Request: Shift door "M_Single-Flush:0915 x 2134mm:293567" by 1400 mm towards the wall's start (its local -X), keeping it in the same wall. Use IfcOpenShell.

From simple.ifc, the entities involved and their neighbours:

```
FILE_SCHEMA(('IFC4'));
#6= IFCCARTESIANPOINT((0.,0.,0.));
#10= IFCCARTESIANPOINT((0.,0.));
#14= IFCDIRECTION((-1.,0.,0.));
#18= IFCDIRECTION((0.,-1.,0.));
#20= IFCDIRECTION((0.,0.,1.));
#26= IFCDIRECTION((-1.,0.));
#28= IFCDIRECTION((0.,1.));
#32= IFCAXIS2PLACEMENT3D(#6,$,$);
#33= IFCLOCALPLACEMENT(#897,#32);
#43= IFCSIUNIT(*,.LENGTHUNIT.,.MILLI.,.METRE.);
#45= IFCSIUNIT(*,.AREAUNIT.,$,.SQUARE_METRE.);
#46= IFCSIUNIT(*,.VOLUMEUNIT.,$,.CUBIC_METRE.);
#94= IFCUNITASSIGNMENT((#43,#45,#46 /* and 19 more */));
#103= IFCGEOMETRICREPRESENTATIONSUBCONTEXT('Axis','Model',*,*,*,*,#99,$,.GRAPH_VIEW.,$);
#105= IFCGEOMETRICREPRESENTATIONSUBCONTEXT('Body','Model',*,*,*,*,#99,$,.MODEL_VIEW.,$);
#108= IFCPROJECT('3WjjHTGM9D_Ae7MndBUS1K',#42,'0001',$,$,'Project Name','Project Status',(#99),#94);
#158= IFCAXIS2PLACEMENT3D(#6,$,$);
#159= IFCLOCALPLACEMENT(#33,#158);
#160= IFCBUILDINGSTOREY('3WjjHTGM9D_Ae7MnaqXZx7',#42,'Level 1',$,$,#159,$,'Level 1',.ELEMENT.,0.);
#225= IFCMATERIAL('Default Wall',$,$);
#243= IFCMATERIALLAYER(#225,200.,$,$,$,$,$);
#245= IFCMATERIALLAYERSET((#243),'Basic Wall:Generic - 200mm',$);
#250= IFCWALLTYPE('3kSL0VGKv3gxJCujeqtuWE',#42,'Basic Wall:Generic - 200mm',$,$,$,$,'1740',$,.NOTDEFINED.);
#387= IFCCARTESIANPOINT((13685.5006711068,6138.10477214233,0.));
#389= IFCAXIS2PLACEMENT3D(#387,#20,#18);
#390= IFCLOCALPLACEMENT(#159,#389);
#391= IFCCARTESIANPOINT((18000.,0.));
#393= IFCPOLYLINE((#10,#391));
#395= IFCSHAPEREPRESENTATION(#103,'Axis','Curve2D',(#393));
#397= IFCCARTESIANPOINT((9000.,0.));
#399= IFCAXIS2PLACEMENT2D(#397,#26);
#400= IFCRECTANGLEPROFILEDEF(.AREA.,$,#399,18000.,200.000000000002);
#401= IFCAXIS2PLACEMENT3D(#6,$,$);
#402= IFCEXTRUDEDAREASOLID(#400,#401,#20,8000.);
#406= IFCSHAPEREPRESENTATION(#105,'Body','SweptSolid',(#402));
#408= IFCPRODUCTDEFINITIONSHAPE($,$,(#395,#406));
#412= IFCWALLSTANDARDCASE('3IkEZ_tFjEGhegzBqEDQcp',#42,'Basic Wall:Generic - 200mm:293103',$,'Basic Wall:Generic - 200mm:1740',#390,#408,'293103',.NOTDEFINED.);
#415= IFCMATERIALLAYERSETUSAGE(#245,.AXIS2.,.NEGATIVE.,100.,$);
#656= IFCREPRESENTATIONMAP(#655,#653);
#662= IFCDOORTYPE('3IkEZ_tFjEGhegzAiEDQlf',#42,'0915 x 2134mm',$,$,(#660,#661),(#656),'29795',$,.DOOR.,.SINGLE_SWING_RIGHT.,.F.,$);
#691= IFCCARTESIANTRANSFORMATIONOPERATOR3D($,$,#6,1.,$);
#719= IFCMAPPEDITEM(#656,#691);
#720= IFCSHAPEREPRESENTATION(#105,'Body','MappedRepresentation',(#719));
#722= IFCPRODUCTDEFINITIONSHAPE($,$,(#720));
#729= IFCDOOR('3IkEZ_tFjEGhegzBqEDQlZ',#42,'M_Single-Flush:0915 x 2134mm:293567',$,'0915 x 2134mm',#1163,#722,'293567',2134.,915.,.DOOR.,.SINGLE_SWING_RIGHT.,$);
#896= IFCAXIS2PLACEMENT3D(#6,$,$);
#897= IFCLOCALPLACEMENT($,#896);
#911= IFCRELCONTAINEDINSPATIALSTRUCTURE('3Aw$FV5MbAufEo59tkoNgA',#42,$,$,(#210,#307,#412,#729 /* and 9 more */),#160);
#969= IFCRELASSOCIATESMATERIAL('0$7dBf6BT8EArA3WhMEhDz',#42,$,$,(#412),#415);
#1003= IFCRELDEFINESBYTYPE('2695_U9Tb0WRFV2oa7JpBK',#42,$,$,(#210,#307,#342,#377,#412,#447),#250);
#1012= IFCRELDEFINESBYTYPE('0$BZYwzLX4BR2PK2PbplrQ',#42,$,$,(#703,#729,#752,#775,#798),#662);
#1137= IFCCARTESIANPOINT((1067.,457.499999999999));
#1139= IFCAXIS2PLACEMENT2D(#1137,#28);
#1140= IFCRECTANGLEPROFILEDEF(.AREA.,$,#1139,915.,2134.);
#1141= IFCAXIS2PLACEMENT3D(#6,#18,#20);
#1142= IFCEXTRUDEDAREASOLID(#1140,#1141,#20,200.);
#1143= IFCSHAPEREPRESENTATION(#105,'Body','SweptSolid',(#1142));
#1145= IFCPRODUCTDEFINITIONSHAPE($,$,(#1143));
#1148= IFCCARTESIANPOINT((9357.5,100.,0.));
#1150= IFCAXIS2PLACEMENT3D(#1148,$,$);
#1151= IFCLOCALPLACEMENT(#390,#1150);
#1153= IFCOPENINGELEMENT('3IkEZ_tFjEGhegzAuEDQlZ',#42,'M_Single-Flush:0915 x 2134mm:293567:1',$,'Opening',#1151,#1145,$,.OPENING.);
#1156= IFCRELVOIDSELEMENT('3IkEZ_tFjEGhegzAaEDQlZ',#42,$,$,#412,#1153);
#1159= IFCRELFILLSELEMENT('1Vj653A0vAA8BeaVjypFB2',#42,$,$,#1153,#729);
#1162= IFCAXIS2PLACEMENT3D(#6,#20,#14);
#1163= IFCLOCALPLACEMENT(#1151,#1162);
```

```python
import ifcopenshell
import ifcopenshell.api.geometry
import ifcopenshell.util.placement
import ifcopenshell.util.unit

model = ifcopenshell.open("simple.ifc")
unit_scale = ifcopenshell.util.unit.calculate_unit_scale(model)

door = model.by_id(729)
opening = door.FillsVoids[0].RelatingOpeningElement
wall = opening.VoidsElements[0].RelatingBuildingElement

wall_matrix = ifcopenshell.util.placement.get_local_placement(wall.ObjectPlacement)
shift = wall_matrix[:3, 0] * -1.4 / unit_scale
before = ifcopenshell.util.placement.get_local_placement(door.ObjectPlacement)[:3, 3].copy()

# The door is placed relative to its opening, so it follows when the opening moves.
matrix = ifcopenshell.util.placement.get_local_placement(opening.ObjectPlacement)
matrix[:3, 3] += shift
ifcopenshell.api.geometry.edit_object_placement(
    model, product=opening, matrix=matrix, is_si=False, should_transform_children=True
)

after = ifcopenshell.util.placement.get_local_placement(door.ObjectPlacement)[:3, 3]
print("door moved by", (after - before).round(3) + 0.0)

model.write("simple_v2.ifc")
```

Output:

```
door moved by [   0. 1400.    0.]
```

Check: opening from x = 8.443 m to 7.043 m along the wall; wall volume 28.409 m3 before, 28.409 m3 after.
